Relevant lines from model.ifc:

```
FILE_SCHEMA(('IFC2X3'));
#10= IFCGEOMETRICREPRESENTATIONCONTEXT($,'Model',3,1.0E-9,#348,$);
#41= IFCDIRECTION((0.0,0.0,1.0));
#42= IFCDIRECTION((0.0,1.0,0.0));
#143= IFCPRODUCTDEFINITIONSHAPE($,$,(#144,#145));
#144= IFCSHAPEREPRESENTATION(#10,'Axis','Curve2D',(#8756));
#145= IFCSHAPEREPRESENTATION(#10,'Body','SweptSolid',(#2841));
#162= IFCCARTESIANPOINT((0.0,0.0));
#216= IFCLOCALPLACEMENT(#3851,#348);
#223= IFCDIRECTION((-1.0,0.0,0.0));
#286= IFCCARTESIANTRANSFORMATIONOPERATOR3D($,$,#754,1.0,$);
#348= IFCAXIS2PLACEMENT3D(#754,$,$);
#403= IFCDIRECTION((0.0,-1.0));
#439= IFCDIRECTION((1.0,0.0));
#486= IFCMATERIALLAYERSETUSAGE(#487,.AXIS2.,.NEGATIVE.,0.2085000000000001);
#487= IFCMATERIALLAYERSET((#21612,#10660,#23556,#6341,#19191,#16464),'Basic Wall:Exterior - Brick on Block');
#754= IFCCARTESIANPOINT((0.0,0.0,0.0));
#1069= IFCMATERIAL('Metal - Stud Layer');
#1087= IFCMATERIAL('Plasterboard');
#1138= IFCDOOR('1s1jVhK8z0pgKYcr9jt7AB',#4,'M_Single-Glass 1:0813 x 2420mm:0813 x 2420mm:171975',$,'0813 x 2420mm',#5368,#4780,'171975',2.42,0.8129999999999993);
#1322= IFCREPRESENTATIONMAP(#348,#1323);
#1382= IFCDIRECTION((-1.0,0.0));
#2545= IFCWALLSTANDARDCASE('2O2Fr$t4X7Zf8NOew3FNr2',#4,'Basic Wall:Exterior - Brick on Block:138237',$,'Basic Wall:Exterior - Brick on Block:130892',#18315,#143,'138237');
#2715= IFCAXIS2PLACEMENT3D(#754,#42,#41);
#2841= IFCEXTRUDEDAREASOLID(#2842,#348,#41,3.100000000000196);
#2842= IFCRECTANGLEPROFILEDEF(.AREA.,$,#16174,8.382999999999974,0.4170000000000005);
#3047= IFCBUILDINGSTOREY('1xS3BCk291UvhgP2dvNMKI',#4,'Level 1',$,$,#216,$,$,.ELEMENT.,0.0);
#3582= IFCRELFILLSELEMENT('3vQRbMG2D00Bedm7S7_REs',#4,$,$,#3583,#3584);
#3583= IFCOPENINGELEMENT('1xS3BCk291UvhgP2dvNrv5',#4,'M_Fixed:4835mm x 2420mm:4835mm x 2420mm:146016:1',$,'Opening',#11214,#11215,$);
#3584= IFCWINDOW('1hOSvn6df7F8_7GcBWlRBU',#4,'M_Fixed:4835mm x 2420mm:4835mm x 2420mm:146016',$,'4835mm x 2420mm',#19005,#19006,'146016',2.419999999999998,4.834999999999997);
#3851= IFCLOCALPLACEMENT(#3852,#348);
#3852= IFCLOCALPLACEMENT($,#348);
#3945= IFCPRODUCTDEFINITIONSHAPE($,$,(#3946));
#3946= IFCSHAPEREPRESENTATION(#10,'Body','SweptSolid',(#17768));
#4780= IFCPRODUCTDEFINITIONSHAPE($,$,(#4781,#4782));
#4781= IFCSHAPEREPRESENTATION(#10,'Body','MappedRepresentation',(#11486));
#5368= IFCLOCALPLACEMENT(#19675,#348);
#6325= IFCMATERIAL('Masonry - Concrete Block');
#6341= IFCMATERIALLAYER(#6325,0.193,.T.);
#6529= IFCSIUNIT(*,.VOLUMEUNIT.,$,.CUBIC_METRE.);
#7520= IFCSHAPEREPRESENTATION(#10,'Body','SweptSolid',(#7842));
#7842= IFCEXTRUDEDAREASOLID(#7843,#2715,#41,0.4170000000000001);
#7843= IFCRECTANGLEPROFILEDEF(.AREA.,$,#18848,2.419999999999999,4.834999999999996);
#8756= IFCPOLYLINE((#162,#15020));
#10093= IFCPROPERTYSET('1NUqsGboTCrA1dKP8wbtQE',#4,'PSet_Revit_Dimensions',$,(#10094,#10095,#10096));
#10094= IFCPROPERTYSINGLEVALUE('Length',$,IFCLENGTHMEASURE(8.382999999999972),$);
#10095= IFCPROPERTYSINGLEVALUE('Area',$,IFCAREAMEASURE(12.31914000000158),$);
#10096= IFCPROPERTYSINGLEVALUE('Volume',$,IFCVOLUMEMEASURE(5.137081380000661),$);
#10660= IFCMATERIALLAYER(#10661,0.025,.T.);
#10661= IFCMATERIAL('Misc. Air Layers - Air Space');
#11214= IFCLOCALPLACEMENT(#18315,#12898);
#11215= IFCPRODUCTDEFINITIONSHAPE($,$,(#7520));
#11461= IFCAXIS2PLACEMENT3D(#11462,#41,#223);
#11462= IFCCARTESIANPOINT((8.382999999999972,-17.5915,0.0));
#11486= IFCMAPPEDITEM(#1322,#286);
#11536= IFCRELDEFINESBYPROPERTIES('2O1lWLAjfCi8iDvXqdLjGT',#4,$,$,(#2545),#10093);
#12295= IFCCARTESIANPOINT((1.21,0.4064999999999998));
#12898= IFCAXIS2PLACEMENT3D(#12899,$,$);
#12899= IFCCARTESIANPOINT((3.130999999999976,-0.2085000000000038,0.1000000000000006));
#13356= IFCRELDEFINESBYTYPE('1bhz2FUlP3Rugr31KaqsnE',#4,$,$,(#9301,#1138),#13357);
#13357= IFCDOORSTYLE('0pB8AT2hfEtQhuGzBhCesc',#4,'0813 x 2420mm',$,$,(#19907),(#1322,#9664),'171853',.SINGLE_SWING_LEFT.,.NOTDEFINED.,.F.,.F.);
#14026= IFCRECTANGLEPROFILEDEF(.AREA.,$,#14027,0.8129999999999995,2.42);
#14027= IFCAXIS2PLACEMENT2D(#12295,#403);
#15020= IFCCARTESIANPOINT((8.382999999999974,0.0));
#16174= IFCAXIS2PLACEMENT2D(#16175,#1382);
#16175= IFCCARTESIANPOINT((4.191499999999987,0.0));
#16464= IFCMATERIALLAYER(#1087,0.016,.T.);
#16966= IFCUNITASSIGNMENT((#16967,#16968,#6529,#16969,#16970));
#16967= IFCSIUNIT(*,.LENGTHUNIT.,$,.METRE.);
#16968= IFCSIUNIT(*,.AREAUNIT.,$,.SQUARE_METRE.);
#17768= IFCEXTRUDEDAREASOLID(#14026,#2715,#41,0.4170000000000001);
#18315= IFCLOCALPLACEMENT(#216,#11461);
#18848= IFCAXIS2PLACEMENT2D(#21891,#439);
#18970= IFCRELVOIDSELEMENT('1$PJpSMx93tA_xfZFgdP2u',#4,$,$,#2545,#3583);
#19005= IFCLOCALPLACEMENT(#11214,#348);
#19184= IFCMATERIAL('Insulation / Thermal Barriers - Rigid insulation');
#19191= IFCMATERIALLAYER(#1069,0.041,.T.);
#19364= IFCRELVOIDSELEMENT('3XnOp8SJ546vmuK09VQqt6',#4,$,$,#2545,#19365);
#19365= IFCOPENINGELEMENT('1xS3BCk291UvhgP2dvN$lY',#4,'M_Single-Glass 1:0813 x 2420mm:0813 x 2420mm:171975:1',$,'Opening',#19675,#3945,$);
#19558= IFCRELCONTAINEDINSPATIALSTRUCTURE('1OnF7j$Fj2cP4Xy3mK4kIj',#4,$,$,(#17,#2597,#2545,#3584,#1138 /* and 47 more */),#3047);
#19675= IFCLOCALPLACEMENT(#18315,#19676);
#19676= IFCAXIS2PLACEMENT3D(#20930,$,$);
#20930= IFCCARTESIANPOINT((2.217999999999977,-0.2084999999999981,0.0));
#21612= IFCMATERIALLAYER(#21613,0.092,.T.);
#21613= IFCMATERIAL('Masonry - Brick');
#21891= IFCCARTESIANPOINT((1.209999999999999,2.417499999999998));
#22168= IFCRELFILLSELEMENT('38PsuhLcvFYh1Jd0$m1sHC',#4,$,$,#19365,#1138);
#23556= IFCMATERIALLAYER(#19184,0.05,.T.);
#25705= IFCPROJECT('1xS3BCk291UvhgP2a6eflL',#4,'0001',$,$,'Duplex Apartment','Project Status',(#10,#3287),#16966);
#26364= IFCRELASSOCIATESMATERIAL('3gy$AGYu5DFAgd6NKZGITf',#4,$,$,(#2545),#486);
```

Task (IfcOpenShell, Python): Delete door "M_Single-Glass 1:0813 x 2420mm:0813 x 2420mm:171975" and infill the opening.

```python
import ifcopenshell
import ifcopenshell.api.feature
import ifcopenshell.api.pset
import ifcopenshell.api.root
import ifcopenshell.geom
import ifcopenshell.util.element
import ifcopenshell.util.shape
import ifcopenshell.util.unit

model = ifcopenshell.open("model.ifc")
area_scale = ifcopenshell.util.unit.calculate_unit_scale(model, "AREAUNIT")
volume_scale = ifcopenshell.util.unit.calculate_unit_scale(model, "VOLUMEUNIT")
settings = ifcopenshell.geom.settings()


def volume(element):
    """Net volume in cubic metres, openings subtracted."""
    shape = ifcopenshell.geom.create_shape(settings, element)
    return ifcopenshell.util.shape.get_volume(shape.geometry)


door = model.by_guid("1s1jVhK8z0pgKYcr9jt7AB")
opening = door.FillsVoids[0].RelatingOpeningElement
wall = opening.VoidsElements[0].RelatingBuildingElement
before = volume(wall)

ifcopenshell.api.root.remove_product(model, product=door)
ifcopenshell.api.feature.remove_feature(model, feature=opening)

after = volume(wall)
thickness = 0.417  # wall thickness in metres

# Update the wall's stored quantities.
pset = model.by_id(ifcopenshell.util.element.get_pset(wall, "PSet_Revit_Dimensions", should_inherit=False)["id"])
ifcopenshell.api.pset.edit_pset(model, pset=pset, properties={
    "Area": model.create_entity("IfcAreaMeasure", after / thickness / area_scale),
    "Volume": model.create_entity("IfcVolumeMeasure", after / volume_scale),
})

print(f"wall volume {before:.3f} -> {after:.3f} m3")

model.write("model_edited.ifc")
```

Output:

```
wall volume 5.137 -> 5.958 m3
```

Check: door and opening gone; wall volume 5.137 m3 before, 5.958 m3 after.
